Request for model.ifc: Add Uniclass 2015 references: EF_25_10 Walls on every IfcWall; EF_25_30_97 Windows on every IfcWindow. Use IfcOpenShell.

First a look at what the model holds.

```python
import ifcopenshell

model = ifcopenshell.open("model.ifc")
print(model.schema)
print("classifications:", [c.Name for c in model.by_type("IfcClassification")])
for ifc_class in ("IfcDoor", "IfcRoof", "IfcStair", "IfcWall", "IfcWindow"):
    print(ifc_class, len(model.by_type(ifc_class)))
```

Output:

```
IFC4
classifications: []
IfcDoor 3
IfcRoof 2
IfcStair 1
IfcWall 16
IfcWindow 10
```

```python
import ifcopenshell
import ifcopenshell.api.classification

model = ifcopenshell.open("model.ifc")

system = ifcopenshell.api.classification.add_classification(model, classification="Uniclass 2015")

codes = {
    "IfcWall": ("EF_25_10", "Walls"),
    "IfcWindow": ("EF_25_30_97", "Windows"),
}
for ifc_class, (code, name) in codes.items():
    products = model.by_type(ifc_class)
    ifcopenshell.api.classification.add_reference(
        model, products=products, classification=system, identification=code, name=name
    )
    print(code, len(products))

model.write("model_v2.ifc")
```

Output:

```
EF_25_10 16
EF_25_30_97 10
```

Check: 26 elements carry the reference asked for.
